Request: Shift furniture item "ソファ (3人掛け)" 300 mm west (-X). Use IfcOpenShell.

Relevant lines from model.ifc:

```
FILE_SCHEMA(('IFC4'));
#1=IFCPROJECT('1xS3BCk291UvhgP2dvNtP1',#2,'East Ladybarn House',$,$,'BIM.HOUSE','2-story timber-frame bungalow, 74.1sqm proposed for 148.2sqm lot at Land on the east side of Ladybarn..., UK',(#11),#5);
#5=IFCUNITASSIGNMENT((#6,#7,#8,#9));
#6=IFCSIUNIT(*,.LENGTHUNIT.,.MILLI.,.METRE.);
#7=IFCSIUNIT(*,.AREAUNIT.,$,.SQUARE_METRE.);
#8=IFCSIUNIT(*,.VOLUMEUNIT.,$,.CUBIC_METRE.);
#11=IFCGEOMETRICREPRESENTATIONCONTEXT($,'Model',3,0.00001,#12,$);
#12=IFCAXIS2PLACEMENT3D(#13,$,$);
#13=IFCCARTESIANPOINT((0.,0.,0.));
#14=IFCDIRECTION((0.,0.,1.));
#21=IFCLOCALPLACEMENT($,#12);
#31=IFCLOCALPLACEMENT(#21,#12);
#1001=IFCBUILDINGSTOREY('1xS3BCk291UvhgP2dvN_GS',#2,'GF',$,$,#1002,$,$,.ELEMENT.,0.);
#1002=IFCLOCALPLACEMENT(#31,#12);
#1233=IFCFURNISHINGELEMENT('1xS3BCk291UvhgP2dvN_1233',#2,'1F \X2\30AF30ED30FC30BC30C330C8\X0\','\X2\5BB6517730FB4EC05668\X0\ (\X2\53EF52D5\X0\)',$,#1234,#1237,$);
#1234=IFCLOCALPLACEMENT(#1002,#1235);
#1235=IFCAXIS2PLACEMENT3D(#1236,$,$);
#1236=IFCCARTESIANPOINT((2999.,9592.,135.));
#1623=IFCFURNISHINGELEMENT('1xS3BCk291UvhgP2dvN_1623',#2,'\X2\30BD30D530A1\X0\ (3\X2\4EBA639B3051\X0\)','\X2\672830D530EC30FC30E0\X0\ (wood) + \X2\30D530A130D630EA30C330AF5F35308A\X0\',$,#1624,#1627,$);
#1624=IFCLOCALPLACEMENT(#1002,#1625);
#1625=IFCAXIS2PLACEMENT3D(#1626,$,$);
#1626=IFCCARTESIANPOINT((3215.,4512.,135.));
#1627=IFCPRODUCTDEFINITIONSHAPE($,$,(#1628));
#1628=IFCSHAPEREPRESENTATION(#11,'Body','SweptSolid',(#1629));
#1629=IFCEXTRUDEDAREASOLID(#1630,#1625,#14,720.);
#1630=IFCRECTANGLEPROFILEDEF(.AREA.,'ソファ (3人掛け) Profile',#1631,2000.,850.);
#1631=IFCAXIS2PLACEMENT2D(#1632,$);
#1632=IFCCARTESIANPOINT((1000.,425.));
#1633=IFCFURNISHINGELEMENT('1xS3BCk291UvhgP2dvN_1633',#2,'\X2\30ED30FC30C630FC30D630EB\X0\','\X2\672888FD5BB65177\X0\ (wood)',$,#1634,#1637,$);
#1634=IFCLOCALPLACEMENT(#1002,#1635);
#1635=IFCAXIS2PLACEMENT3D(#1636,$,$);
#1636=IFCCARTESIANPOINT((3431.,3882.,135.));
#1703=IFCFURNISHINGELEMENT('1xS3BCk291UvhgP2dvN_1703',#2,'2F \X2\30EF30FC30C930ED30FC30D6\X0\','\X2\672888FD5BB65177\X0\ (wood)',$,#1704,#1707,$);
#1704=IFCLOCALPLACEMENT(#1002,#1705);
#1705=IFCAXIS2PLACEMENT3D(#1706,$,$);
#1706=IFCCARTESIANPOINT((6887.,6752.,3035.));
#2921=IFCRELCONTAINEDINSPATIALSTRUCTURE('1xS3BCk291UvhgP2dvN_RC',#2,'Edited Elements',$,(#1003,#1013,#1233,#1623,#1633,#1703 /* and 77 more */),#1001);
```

```python
import ifcopenshell
import ifcopenshell.api.geometry
import ifcopenshell.util.placement
import ifcopenshell.util.unit

model = ifcopenshell.open("model.ifc")
unit_scale = ifcopenshell.util.unit.calculate_unit_scale(model)

item = model.by_guid("1xS3BCk291UvhgP2dvN_1623")
matrix = ifcopenshell.util.placement.get_local_placement(item.ObjectPlacement)
matrix[0, 3] -= 0.3 / unit_scale
ifcopenshell.api.geometry.edit_object_placement(model, product=item, matrix=matrix, is_si=False)

print(ifcopenshell.util.placement.get_local_placement(item.ObjectPlacement).round(3) + 0.0)

model.write("model_rev.ifc")
```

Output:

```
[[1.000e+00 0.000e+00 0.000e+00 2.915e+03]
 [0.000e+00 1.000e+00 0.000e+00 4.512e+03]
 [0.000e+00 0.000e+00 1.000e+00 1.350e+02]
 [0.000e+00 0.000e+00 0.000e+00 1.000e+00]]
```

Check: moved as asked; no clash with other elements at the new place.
